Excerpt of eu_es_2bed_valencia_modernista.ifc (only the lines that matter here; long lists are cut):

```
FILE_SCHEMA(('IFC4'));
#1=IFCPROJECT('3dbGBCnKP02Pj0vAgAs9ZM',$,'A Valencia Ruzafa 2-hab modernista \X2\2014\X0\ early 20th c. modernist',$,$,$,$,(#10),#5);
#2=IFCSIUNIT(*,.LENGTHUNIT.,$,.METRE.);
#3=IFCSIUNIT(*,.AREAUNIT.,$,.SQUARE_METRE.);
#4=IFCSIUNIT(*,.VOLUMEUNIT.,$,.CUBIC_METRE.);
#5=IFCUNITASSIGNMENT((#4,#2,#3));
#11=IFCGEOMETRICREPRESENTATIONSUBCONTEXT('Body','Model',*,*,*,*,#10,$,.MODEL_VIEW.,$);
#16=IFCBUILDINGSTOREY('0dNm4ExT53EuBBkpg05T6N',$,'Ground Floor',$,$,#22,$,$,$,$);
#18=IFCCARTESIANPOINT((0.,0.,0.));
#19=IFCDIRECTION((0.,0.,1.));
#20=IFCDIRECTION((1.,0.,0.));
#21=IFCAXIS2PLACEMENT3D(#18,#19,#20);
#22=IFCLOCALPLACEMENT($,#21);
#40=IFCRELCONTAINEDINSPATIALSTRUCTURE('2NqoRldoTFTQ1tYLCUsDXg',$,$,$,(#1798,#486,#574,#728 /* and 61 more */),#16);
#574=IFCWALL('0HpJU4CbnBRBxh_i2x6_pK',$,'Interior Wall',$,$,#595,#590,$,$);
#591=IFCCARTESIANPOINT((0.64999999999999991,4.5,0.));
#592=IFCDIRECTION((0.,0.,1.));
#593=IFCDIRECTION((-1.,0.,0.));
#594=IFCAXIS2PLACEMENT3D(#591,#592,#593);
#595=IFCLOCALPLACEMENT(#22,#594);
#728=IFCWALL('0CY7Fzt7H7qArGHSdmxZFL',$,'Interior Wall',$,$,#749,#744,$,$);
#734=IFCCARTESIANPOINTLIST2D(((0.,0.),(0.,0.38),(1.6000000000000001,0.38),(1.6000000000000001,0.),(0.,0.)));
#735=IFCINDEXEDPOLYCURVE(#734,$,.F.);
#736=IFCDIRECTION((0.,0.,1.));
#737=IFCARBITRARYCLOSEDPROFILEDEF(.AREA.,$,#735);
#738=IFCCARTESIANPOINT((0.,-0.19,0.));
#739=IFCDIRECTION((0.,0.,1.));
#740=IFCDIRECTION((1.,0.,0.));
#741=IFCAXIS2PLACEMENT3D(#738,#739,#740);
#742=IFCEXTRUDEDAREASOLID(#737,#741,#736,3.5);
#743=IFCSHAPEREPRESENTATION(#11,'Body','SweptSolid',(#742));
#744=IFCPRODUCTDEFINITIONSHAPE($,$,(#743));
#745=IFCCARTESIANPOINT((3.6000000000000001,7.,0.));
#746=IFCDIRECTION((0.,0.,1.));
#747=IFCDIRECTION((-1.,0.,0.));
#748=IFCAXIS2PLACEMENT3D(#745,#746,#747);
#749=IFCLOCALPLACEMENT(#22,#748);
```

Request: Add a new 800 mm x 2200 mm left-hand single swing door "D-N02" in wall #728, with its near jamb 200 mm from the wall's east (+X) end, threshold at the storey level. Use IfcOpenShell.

```python
import numpy as np
import ifcopenshell
import ifcopenshell.api.feature
import ifcopenshell.api.geometry
import ifcopenshell.api.root
import ifcopenshell.api.spatial
import ifcopenshell.geom
import ifcopenshell.util.element
import ifcopenshell.util.placement
import ifcopenshell.util.representation
import ifcopenshell.util.shape
import ifcopenshell.util.unit

model = ifcopenshell.open("eu_es_2bed_valencia_modernista.ifc")
unit_scale = ifcopenshell.util.unit.calculate_unit_scale(model)
settings = ifcopenshell.geom.settings()


def volume(element):
    """Net volume in cubic metres, openings subtracted."""
    shape = ifcopenshell.geom.create_shape(settings, element)
    return ifcopenshell.util.shape.get_volume(shape.geometry)


wall = model.by_guid("0CY7Fzt7H7qArGHSdmxZFL")
storey = ifcopenshell.util.element.get_container(wall, ifc_class="IfcBuildingStorey")
context = ifcopenshell.util.representation.get_context(model, "Model", "Body", "MODEL_VIEW")
before = volume(wall)

width, height, from_end, sill = 0.8, 2.2, 0.2, 0.0  # metres

# The wall runs along its own X axis, and the end named is its -X end.
wall_shape = ifcopenshell.geom.create_shape(settings, wall)
x, y, z = ifcopenshell.util.shape.get_vertices(wall_shape.geometry).T
start = x.min() + from_end
face, thickness = float(y.min()), float(y.max() - y.min())
wall_matrix = ifcopenshell.util.placement.get_local_placement(wall.ObjectPlacement)
level = ifcopenshell.util.placement.get_local_placement(storey.ObjectPlacement)[2, 3]


def in_wall(x, y):
    """Placement at x, y metres in the wall's axes, at sill height."""
    matrix = wall_matrix.copy()
    matrix[:, 3] = wall_matrix @ np.array([x / unit_scale, y / unit_scale, 0.0, 1.0])
    matrix[2, 3] = level + sill / unit_scale
    return matrix


# Opening: a box that overshoots both wall faces by 50 mm.
opening = ifcopenshell.api.root.create_entity(model, ifc_class="IfcOpeningElement", predefined_type="OPENING")
box = ifcopenshell.api.geometry.add_wall_representation(
    model, context=context, length=width, height=height, thickness=thickness + 0.1
)
ifcopenshell.api.geometry.assign_representation(model, product=opening, representation=box)
ifcopenshell.api.geometry.edit_object_placement(model, product=opening, matrix=in_wall(start, face - 0.05), is_si=False)
ifcopenshell.api.feature.add_feature(model, feature=opening, element=wall)

door = ifcopenshell.api.root.create_entity(model, ifc_class="IfcDoor", name="D-N02", predefined_type="DOOR")
door.OverallWidth, door.OverallHeight = width / unit_scale, height / unit_scale
door.OperationType = "SINGLE_SWING_LEFT"
body = ifcopenshell.api.geometry.add_door_representation(
    model,
    context=context,
    overall_width=door.OverallWidth,
    overall_height=door.OverallHeight,
    operation_type="SINGLE_SWING_LEFT",
    lining_properties={"LiningDepth": thickness / unit_scale, "ThresholdDepth": thickness / unit_scale},
)
ifcopenshell.api.geometry.assign_representation(model, product=door, representation=body)
ifcopenshell.api.spatial.assign_container(model, products=[door], relating_structure=storey)
ifcopenshell.api.feature.add_filling(model, opening=opening, element=door)

# The lining spans the wall, so the door starts at the wall face.
ifcopenshell.api.geometry.edit_object_placement(model, product=door, matrix=in_wall(start, face), is_si=False)

after = volume(wall)

print(f"wall volume {before:.3f} -> {after:.3f} m3")

model.write("eu_es_2bed_valencia_modernista-out.ifc")
```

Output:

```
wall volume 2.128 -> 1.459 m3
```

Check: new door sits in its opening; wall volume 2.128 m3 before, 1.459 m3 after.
